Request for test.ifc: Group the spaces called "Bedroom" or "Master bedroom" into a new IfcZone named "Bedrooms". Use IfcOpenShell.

First a look at what the model holds.

```python
import ifcopenshell

model = ifcopenshell.open("test.ifc")
print(model.schema)
seen = {}
for space in model.by_type("IfcSpace"):
    seen[space.LongName] = seen.get(space.LongName, 0) + 1
for name, count in sorted(seen.items(), key=str):
    print(count, "x", name)
print("zones:", [z.Name for z in model.by_type("IfcZone")][:20])
```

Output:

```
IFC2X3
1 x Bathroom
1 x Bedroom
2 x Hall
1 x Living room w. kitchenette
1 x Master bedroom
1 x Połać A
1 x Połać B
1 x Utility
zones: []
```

```python
import ifcopenshell
import ifcopenshell.api.group
import ifcopenshell.api.root

model = ifcopenshell.open("test.ifc")

names = {"Bedroom", "Master bedroom"}
spaces = [s for s in model.by_type("IfcSpace") if s.LongName in names]

zone = ifcopenshell.api.root.create_entity(model, ifc_class="IfcZone", name="Bedrooms")
ifcopenshell.api.group.assign_group(model, products=spaces, group=zone)
print(len(spaces), "spaces in", zone.Name)

model.write("test_v2.ifc")
```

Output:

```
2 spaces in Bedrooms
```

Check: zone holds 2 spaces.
